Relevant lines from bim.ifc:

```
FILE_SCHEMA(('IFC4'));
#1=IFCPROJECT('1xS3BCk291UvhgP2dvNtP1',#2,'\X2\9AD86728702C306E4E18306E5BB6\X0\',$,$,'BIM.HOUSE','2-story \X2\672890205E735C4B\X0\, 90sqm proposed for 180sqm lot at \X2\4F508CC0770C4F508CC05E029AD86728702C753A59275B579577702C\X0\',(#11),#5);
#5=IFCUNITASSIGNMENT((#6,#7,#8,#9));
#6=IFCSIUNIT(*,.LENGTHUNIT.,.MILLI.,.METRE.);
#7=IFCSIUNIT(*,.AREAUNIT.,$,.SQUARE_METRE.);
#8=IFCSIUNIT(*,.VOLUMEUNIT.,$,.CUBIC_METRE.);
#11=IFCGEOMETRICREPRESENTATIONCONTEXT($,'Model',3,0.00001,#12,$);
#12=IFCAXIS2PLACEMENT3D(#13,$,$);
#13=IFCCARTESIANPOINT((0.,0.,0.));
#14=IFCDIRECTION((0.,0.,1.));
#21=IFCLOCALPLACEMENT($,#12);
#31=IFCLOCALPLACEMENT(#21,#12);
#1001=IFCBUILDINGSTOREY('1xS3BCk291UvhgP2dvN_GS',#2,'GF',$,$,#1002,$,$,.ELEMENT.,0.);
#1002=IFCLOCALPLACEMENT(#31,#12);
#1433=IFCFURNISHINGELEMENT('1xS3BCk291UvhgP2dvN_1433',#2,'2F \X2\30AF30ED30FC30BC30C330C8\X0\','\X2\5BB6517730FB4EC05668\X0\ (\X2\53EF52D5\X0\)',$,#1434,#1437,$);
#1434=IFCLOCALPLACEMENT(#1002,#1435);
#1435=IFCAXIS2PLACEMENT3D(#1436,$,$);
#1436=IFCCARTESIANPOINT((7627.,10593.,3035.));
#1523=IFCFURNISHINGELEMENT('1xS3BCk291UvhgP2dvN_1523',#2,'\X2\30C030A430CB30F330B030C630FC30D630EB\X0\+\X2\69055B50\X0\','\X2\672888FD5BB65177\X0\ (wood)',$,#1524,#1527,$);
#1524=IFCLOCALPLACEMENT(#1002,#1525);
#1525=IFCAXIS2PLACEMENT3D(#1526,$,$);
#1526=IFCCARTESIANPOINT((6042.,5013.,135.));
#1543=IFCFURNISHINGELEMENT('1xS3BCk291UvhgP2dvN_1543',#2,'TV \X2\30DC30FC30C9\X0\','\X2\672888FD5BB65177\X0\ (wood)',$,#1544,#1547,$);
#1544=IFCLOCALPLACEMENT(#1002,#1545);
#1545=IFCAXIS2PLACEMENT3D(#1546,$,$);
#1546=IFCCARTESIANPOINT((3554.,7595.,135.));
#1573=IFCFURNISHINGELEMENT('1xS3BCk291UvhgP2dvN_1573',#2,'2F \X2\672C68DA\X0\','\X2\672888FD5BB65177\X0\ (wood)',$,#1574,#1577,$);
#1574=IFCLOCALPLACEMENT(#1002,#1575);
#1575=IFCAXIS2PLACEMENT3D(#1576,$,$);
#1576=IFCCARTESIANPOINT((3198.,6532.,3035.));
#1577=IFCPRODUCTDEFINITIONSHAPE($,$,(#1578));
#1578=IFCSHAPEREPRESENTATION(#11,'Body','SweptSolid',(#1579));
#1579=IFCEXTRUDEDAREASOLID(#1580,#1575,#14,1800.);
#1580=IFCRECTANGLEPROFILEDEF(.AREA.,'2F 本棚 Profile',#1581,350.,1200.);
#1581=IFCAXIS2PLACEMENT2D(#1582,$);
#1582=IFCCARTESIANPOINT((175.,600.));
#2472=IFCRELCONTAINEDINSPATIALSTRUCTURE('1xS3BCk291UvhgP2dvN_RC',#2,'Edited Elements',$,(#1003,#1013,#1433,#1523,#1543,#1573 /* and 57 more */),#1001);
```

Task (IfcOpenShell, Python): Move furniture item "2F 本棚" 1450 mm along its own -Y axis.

```python
import ifcopenshell
import ifcopenshell.api.geometry
import ifcopenshell.util.placement
import ifcopenshell.util.unit

model = ifcopenshell.open("bim.ifc")
unit_scale = ifcopenshell.util.unit.calculate_unit_scale(model)

item = model.by_id(1573)
matrix = ifcopenshell.util.placement.get_local_placement(item.ObjectPlacement)
matrix[:3, 3] -= matrix[:3, 1] * 1.45 / unit_scale
ifcopenshell.api.geometry.edit_object_placement(model, product=item, matrix=matrix, is_si=False)

print(ifcopenshell.util.placement.get_local_placement(item.ObjectPlacement).round(3) + 0.0)

model.write("bim_edited.ifc")
```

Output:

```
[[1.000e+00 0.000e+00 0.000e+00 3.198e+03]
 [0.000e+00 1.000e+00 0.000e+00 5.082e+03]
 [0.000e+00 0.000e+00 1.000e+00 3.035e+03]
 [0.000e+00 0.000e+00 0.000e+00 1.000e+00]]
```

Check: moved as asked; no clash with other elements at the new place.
